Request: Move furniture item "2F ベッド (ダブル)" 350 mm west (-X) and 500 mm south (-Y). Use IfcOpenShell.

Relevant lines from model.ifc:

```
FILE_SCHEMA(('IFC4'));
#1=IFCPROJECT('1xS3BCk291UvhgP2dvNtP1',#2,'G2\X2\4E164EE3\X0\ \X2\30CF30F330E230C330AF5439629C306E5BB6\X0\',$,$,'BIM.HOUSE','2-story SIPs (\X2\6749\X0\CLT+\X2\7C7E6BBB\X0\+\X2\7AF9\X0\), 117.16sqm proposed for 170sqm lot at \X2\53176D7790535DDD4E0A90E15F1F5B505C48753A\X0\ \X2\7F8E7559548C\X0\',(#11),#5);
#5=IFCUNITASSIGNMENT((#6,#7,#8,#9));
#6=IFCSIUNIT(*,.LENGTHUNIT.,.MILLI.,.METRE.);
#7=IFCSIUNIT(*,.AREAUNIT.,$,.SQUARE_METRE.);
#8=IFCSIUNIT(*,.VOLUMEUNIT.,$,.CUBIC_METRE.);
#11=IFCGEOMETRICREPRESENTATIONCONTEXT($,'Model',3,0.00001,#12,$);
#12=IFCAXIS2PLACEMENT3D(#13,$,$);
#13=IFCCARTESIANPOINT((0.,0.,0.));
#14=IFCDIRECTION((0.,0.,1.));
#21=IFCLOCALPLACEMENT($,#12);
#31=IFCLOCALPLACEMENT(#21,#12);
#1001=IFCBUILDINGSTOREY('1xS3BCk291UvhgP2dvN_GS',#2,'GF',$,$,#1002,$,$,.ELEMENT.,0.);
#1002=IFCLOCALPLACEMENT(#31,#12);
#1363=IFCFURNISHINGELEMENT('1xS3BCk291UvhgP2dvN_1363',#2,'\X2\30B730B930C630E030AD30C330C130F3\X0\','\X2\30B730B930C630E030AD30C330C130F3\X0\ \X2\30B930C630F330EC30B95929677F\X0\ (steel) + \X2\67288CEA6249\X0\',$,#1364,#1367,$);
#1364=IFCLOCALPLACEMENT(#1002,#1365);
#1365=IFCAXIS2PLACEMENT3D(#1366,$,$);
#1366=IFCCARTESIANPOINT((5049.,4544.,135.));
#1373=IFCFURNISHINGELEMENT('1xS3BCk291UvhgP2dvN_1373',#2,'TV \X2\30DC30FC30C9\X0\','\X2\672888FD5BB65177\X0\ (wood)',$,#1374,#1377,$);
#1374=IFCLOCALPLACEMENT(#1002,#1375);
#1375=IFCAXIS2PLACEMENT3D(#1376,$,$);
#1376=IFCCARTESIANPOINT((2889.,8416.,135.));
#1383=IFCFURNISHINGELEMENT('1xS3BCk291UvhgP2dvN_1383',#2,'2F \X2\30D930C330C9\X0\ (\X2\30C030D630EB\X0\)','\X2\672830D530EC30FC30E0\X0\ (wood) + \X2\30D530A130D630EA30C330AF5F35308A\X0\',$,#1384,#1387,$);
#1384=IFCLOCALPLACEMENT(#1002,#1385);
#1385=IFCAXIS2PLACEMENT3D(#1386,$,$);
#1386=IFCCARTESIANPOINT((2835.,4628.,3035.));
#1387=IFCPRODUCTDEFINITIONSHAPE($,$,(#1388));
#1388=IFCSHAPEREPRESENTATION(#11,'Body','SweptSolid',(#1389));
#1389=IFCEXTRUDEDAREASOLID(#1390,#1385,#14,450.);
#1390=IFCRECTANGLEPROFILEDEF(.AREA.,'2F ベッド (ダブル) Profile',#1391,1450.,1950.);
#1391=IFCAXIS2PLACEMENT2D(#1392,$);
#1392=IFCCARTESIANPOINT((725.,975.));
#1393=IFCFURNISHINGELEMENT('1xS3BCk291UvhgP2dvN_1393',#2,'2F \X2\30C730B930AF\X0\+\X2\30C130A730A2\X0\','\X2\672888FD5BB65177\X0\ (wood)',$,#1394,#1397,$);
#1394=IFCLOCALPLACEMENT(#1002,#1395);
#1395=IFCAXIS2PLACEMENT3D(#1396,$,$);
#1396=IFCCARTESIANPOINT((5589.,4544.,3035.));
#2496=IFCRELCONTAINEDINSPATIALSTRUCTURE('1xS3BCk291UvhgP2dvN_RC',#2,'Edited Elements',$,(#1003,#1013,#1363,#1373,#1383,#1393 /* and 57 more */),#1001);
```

```python
import ifcopenshell
import ifcopenshell.api.geometry
import ifcopenshell.util.placement
import ifcopenshell.util.unit

model = ifcopenshell.open("model.ifc")
unit_scale = ifcopenshell.util.unit.calculate_unit_scale(model)

item = model.by_id(1383)
matrix = ifcopenshell.util.placement.get_local_placement(item.ObjectPlacement)
matrix[0, 3] -= 0.35 / unit_scale
matrix[1, 3] -= 0.5 / unit_scale
ifcopenshell.api.geometry.edit_object_placement(model, product=item, matrix=matrix, is_si=False)

print(ifcopenshell.util.placement.get_local_placement(item.ObjectPlacement).round(3) + 0.0)

model.write("model_updated.ifc")
```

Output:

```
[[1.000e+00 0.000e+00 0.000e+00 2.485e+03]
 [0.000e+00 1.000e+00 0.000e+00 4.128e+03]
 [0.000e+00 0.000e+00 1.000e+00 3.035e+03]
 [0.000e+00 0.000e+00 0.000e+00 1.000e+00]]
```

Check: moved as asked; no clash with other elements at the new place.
